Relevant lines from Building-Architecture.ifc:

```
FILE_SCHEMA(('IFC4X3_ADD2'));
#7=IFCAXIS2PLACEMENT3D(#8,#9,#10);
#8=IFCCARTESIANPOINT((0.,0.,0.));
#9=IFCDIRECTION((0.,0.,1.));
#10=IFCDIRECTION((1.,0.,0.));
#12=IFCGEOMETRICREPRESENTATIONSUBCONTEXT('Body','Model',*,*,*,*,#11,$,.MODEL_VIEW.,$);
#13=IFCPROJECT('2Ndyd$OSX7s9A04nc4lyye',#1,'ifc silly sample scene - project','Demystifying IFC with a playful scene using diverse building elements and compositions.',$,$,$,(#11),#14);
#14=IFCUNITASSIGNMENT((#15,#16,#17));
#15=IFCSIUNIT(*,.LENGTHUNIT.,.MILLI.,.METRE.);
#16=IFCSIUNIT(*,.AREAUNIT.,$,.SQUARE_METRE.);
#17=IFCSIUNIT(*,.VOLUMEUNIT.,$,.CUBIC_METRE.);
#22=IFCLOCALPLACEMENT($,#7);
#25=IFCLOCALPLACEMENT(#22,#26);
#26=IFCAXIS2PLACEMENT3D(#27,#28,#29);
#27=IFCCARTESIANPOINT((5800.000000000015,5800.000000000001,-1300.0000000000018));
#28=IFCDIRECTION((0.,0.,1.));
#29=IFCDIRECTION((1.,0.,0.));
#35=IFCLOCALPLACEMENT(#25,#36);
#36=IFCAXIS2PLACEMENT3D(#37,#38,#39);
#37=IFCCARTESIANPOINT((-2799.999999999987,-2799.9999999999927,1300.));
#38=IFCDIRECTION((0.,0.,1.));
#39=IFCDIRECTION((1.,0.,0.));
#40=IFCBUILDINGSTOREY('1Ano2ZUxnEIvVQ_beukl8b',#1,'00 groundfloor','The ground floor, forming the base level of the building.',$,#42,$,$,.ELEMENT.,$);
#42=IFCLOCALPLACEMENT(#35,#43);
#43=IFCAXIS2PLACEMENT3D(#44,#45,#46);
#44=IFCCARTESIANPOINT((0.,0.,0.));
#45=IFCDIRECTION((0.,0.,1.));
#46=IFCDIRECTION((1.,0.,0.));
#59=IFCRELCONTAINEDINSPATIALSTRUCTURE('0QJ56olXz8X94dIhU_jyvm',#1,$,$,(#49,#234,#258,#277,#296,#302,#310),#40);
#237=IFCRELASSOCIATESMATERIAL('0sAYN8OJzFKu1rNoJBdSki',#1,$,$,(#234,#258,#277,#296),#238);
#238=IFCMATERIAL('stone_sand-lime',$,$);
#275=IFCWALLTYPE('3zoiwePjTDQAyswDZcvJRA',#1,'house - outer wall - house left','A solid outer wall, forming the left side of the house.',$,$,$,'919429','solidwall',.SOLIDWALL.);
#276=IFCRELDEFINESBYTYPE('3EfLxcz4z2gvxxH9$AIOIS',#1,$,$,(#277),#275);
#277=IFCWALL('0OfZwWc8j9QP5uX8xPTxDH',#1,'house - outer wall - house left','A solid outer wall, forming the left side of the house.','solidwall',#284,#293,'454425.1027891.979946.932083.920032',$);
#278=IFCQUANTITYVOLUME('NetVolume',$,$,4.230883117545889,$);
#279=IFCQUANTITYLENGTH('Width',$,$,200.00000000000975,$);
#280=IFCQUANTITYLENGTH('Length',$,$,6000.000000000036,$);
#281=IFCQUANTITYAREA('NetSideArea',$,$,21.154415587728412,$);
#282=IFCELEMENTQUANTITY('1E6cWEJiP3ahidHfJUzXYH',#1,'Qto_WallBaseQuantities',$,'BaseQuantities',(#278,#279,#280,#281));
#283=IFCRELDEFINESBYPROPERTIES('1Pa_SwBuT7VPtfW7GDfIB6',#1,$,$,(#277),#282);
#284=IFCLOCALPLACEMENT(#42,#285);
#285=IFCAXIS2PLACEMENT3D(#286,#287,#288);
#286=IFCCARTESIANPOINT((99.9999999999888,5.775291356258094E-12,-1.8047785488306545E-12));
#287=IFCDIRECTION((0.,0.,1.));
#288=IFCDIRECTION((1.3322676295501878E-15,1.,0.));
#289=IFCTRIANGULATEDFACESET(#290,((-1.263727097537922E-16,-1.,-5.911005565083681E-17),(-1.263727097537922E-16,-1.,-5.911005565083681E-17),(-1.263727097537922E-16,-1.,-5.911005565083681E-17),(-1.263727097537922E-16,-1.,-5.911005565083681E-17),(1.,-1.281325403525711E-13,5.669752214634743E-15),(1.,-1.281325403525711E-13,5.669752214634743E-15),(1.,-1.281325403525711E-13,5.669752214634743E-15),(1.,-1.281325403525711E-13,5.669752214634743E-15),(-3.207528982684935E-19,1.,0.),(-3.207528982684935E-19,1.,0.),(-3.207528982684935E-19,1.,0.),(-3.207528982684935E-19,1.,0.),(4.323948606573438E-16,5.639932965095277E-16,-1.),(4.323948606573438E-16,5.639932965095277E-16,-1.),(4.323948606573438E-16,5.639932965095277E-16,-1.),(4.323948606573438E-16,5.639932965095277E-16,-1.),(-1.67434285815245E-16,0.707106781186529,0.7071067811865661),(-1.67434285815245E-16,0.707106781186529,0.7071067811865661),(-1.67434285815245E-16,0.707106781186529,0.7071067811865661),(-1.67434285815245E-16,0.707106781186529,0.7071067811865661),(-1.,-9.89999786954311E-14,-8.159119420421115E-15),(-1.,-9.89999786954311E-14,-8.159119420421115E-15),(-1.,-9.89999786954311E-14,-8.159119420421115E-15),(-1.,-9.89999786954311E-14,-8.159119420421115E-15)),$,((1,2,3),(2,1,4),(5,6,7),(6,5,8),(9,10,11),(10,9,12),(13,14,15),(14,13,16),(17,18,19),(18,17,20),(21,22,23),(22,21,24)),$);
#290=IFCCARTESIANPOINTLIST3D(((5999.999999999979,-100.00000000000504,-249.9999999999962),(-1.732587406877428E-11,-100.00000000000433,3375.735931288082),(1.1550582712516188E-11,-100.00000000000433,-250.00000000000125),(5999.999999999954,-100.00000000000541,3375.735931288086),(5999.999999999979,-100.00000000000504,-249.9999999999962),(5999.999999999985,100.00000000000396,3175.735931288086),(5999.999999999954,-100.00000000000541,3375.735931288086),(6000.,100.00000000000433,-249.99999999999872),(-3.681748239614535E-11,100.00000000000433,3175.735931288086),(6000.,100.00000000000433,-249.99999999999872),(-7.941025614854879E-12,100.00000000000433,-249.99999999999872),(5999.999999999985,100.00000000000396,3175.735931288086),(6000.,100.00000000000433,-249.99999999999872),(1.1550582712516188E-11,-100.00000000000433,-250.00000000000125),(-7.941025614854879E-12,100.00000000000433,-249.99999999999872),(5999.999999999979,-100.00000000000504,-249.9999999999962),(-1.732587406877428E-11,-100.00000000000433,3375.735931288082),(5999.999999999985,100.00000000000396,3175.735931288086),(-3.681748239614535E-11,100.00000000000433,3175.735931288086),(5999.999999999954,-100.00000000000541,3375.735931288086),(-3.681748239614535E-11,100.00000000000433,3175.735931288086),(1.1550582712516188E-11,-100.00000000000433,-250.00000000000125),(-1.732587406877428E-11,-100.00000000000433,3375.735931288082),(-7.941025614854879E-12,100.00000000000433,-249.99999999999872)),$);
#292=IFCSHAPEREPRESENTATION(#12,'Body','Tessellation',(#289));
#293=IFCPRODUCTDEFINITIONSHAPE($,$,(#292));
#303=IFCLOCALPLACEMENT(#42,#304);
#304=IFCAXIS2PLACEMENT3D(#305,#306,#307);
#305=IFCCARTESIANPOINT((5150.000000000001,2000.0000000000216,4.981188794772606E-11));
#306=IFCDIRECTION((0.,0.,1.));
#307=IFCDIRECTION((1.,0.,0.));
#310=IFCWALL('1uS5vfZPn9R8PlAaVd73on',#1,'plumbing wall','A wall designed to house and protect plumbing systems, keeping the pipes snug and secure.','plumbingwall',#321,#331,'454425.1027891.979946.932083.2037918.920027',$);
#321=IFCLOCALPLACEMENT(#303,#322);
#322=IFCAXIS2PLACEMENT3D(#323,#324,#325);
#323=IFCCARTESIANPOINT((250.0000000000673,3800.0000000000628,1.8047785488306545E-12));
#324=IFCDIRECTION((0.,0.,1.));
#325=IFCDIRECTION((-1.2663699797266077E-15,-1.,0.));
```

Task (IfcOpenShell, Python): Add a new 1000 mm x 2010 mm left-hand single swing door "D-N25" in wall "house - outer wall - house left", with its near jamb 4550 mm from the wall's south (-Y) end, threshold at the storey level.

```python
import numpy as np
import ifcopenshell
import ifcopenshell.api.feature
import ifcopenshell.api.geometry
import ifcopenshell.api.pset
import ifcopenshell.api.root
import ifcopenshell.api.spatial
import ifcopenshell.geom
import ifcopenshell.util.element
import ifcopenshell.util.placement
import ifcopenshell.util.representation
import ifcopenshell.util.shape
import ifcopenshell.util.unit

model = ifcopenshell.open("Building-Architecture.ifc")
unit_scale = ifcopenshell.util.unit.calculate_unit_scale(model)
area_scale = ifcopenshell.util.unit.calculate_unit_scale(model, "AREAUNIT")
volume_scale = ifcopenshell.util.unit.calculate_unit_scale(model, "VOLUMEUNIT")
settings = ifcopenshell.geom.settings()


def volume(element):
    """Net volume in cubic metres, openings subtracted."""
    shape = ifcopenshell.geom.create_shape(settings, element)
    return ifcopenshell.util.shape.get_volume(shape.geometry)


wall = model.by_guid("0OfZwWc8j9QP5uX8xPTxDH")
storey = ifcopenshell.util.element.get_container(wall, ifc_class="IfcBuildingStorey")
context = ifcopenshell.util.representation.get_context(model, "Model", "Body", "MODEL_VIEW")
before = volume(wall)

width, height, from_end, sill = 1, 2.01, 4.55, 0.0  # metres

# The wall runs along its own X axis, and the end named is its -X end.
wall_shape = ifcopenshell.geom.create_shape(settings, wall)
x, y, z = ifcopenshell.util.shape.get_vertices(wall_shape.geometry).T
start = x.min() + from_end
face, thickness = float(y.min()), float(y.max() - y.min())
wall_matrix = ifcopenshell.util.placement.get_local_placement(wall.ObjectPlacement)
level = ifcopenshell.util.placement.get_local_placement(storey.ObjectPlacement)[2, 3]


def in_wall(x, y):
    """Placement at x, y metres in the wall's axes, at sill height."""
    matrix = wall_matrix.copy()
    matrix[:, 3] = wall_matrix @ np.array([x / unit_scale, y / unit_scale, 0.0, 1.0])
    matrix[2, 3] = level + sill / unit_scale
    return matrix


# Opening: a box that overshoots both wall faces by 50 mm.
opening = ifcopenshell.api.root.create_entity(model, ifc_class="IfcOpeningElement", predefined_type="OPENING")
box = ifcopenshell.api.geometry.add_wall_representation(
    model, context=context, length=width, height=height, thickness=thickness + 0.1
)
ifcopenshell.api.geometry.assign_representation(model, product=opening, representation=box)
ifcopenshell.api.geometry.edit_object_placement(model, product=opening, matrix=in_wall(start, face - 0.05), is_si=False)
ifcopenshell.api.feature.add_feature(model, feature=opening, element=wall)

door = ifcopenshell.api.root.create_entity(model, ifc_class="IfcDoor", name="D-N25", predefined_type="DOOR")
door.OverallWidth, door.OverallHeight = width / unit_scale, height / unit_scale
door.OperationType = "SINGLE_SWING_LEFT"
body = ifcopenshell.api.geometry.add_door_representation(
    model,
    context=context,
    overall_width=door.OverallWidth,
    overall_height=door.OverallHeight,
    operation_type="SINGLE_SWING_LEFT",
    lining_properties={"LiningDepth": thickness / unit_scale, "ThresholdDepth": thickness / unit_scale},
)
ifcopenshell.api.geometry.assign_representation(model, product=door, representation=body)
ifcopenshell.api.spatial.assign_container(model, products=[door], relating_structure=storey)
ifcopenshell.api.feature.add_filling(model, opening=opening, element=door)

# The lining spans the wall, so the door starts at the wall face.
ifcopenshell.api.geometry.edit_object_placement(model, product=door, matrix=in_wall(start, face), is_si=False)

after = volume(wall)

# Update the wall's stored quantities.
qto = model.by_id(ifcopenshell.util.element.get_pset(wall, "Qto_WallBaseQuantities", should_inherit=False)["id"])
ifcopenshell.api.pset.edit_qto(model, qto=qto, properties={
    "NetVolume": after / volume_scale,
    "NetSideArea": after / thickness / area_scale,
})

print(f"wall volume {before:.3f} -> {after:.3f} m3")

model.write("Building-Architecture_v2.ifc")
```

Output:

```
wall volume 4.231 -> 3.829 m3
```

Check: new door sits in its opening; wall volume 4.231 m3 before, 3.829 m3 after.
